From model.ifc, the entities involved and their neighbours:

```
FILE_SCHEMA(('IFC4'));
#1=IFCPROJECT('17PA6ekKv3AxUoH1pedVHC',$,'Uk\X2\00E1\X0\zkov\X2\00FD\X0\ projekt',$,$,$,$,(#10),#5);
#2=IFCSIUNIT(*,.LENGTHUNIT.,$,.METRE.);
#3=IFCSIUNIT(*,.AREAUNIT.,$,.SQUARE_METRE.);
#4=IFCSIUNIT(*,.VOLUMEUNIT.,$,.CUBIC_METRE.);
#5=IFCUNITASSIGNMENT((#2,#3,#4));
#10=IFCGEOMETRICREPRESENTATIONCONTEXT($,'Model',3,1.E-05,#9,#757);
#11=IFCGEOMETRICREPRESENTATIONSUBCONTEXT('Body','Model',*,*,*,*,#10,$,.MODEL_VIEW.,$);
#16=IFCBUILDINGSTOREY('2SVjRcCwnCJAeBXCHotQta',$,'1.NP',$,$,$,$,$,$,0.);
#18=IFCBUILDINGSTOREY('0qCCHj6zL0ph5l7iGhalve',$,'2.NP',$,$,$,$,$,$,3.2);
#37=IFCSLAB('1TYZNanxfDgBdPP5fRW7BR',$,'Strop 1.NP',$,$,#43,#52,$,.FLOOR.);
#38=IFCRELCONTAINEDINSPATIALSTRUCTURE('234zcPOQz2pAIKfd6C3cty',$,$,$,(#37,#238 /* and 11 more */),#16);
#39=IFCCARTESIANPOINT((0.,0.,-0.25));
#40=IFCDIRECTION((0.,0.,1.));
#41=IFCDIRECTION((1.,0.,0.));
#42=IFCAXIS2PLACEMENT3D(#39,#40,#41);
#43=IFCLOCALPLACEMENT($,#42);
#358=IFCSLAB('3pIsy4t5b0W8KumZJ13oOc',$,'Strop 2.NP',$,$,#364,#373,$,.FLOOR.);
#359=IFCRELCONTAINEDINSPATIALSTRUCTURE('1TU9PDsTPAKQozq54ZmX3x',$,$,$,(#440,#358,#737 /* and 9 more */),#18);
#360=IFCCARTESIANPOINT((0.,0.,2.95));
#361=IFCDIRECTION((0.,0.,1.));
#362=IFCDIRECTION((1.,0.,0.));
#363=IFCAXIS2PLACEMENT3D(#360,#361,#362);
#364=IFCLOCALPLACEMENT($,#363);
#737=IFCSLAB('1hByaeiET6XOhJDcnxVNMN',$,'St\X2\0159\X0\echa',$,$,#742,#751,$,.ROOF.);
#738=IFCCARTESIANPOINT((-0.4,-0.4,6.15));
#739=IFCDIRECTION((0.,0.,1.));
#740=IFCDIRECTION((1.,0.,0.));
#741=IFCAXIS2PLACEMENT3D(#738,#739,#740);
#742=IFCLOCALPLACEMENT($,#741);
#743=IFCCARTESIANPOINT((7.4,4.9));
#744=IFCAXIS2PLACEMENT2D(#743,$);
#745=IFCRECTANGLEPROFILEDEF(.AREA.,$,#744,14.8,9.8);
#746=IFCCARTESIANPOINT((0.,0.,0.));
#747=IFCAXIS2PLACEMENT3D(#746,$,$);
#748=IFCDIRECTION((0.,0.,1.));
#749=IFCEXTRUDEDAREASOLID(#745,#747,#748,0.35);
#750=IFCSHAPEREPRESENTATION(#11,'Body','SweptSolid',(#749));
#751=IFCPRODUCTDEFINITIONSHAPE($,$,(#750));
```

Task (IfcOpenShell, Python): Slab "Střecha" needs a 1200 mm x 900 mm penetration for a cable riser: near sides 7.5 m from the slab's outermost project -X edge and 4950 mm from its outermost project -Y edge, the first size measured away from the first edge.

```python
import numpy as np
import ifcopenshell
import ifcopenshell.api.feature
import ifcopenshell.api.geometry
import ifcopenshell.api.root
import ifcopenshell.geom
import ifcopenshell.util.placement
import ifcopenshell.util.representation
import ifcopenshell.util.shape
import ifcopenshell.util.unit

model = ifcopenshell.open("model.ifc")
unit_scale = ifcopenshell.util.unit.calculate_unit_scale(model)
settings = ifcopenshell.geom.settings()


def volume(element):
    """Net volume in cubic metres, openings subtracted."""
    shape = ifcopenshell.geom.create_shape(settings, element)
    return ifcopenshell.util.shape.get_volume(shape.geometry)


slab = model.by_guid("1hByaeiET6XOhJDcnxVNMN")
before = volume(slab)

# Extent in the slab's own axes, in metres. The edges named are its -X and -Y sides.
slab_shape = ifcopenshell.geom.create_shape(settings, slab)
vertices = ifcopenshell.util.shape.get_vertices(slab_shape.geometry)
x_min, y_min, bottom = vertices.min(axis=0)
top = vertices[:, 2].max()

opening = ifcopenshell.api.root.create_entity(model, ifc_class="IfcOpeningElement", name="Cable riser opening", predefined_type="OPENING")
context = ifcopenshell.util.representation.get_context(model, "Model", "Body", "MODEL_VIEW")
width, depth = 1.2, 0.9
outline = [(0.0, 0.0), (width, 0.0), (width, depth), (0.0, depth), (0.0, 0.0)]
# Overshoot both faces by 50 mm so the cut is clean.
shape = ifcopenshell.api.geometry.add_slab_representation(
    model, context=context, depth=top - bottom + 0.1, polyline=outline
)
ifcopenshell.api.geometry.assign_representation(model, product=opening, representation=shape)

matrix = ifcopenshell.util.placement.get_local_placement(slab.ObjectPlacement)
matrix[:, 3] = matrix @ np.append(np.array([x_min + 7.5, y_min + 4.95, bottom - 0.05]) / unit_scale, 1.0)
ifcopenshell.api.geometry.edit_object_placement(model, product=opening, matrix=matrix, is_si=False)
ifcopenshell.api.feature.add_feature(model, feature=opening, element=slab)

after = volume(slab)

print(f"slab volume {before:.3f} -> {after:.3f} m3")

model.write("model-out.ifc")
```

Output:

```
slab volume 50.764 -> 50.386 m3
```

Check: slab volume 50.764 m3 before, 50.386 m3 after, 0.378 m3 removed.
